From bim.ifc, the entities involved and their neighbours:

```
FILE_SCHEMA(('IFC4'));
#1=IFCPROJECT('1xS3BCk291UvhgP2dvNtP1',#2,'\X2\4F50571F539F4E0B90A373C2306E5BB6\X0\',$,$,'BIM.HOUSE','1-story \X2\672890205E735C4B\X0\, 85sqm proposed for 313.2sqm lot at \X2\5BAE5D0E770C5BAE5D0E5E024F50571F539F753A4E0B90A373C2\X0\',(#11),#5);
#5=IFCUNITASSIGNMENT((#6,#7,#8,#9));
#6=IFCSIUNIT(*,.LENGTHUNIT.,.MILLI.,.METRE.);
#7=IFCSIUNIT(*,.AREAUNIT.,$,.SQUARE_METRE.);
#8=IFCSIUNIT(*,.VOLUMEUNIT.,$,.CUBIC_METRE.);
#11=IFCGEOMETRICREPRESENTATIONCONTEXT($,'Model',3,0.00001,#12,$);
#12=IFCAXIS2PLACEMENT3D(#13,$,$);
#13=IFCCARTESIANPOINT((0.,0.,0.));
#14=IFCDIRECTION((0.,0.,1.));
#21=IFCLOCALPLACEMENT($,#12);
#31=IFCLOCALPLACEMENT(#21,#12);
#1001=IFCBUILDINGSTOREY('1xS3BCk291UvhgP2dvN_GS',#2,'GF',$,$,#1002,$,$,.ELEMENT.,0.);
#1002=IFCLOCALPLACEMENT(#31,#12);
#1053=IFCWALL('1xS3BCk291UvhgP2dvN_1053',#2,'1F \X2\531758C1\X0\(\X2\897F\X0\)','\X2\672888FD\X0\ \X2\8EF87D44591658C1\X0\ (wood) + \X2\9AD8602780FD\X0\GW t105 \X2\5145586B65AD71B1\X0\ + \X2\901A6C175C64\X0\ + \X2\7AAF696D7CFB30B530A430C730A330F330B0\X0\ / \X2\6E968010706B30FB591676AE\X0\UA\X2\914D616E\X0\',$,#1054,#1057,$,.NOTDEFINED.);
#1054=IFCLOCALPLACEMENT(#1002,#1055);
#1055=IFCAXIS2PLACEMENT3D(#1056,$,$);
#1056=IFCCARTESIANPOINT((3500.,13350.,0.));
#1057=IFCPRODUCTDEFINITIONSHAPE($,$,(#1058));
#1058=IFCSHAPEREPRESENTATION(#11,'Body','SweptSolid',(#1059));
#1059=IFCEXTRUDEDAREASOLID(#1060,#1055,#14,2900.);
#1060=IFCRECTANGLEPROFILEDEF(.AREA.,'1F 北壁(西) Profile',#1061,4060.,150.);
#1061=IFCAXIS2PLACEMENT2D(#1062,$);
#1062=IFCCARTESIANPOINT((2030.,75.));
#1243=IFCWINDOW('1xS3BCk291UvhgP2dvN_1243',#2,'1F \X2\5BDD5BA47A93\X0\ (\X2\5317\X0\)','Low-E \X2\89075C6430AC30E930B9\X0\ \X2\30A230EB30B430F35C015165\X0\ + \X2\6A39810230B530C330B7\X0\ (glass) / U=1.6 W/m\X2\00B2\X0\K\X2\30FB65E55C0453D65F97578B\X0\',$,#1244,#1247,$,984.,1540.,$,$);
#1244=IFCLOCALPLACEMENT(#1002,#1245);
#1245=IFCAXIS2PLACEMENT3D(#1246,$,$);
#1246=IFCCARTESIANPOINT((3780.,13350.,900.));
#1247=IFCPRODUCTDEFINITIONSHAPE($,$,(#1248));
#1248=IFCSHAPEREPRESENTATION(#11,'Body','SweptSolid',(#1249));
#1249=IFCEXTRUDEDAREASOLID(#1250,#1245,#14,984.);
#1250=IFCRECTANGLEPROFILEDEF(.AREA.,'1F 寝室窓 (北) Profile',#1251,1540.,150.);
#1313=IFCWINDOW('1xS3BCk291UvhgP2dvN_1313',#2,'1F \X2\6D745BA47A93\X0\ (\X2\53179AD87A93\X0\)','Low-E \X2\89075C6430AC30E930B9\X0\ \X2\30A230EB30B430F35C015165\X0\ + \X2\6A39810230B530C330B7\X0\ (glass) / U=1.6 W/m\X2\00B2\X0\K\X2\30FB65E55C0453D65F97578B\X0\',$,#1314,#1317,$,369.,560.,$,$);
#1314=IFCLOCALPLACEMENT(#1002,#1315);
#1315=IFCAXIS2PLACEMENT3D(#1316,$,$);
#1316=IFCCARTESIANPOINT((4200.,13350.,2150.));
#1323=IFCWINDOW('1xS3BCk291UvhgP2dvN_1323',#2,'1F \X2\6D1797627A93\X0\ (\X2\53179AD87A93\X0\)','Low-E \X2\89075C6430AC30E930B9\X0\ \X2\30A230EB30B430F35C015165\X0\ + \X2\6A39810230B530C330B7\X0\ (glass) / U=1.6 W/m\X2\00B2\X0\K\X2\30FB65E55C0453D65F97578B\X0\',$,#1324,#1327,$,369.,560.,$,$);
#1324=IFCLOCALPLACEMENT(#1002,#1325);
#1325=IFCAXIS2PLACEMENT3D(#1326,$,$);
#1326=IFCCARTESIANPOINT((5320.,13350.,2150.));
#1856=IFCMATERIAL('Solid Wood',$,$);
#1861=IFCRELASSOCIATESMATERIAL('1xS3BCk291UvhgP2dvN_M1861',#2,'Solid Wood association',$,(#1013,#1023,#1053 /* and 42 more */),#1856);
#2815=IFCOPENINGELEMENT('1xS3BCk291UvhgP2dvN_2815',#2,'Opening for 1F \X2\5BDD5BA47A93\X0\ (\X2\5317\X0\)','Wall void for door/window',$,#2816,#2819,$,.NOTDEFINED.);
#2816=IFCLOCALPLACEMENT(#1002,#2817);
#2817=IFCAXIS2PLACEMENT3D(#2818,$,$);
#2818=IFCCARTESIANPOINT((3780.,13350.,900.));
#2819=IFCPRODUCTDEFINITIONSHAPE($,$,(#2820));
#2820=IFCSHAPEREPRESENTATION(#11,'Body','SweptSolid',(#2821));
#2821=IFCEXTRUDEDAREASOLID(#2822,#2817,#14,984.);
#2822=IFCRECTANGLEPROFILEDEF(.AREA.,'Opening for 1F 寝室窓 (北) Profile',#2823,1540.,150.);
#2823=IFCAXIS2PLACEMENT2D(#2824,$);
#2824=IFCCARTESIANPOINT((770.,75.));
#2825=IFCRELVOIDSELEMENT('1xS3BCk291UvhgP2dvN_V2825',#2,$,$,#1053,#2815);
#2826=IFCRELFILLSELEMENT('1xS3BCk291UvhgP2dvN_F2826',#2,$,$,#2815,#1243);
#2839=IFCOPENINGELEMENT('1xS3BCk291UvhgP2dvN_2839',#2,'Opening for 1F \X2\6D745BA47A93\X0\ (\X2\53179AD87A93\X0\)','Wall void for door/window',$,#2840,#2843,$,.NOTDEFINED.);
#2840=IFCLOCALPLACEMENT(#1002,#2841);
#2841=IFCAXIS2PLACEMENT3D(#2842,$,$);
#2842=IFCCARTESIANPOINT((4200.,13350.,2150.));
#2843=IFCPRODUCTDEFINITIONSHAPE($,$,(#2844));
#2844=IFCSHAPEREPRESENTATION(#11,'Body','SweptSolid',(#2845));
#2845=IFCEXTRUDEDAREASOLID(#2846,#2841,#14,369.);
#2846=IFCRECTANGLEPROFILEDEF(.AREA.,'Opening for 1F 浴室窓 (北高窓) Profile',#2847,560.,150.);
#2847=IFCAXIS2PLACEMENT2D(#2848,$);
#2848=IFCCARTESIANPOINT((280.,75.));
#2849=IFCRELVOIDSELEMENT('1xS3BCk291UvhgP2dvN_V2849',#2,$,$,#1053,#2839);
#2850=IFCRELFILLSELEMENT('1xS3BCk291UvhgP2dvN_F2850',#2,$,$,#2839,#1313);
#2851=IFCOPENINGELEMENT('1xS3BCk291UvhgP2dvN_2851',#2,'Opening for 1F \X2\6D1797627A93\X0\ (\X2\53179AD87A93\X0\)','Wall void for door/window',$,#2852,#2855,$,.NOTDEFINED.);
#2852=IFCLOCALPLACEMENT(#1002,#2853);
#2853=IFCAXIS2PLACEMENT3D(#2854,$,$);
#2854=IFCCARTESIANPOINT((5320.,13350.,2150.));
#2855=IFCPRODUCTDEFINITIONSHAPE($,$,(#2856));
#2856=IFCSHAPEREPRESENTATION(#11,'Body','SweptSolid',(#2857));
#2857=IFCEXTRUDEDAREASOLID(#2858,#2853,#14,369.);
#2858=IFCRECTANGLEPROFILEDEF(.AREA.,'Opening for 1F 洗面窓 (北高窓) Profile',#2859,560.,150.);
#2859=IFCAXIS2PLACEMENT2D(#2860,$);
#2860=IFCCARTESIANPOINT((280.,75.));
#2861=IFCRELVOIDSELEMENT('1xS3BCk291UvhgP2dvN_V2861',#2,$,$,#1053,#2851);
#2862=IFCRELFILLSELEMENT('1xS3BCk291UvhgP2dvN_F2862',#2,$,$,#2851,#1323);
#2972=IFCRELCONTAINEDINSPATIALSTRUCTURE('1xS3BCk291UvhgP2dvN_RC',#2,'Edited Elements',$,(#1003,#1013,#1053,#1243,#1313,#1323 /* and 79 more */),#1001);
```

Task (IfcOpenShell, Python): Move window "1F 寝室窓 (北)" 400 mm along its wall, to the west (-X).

```python
import ifcopenshell
import ifcopenshell.api.geometry
import ifcopenshell.util.placement

model = ifcopenshell.open("bim.ifc")

window = model.by_guid("1xS3BCk291UvhgP2dvN_1243")
opening = window.FillsVoids[0].RelatingOpeningElement
wall = opening.VoidsElements[0].RelatingBuildingElement

wall_matrix = ifcopenshell.util.placement.get_local_placement(wall.ObjectPlacement)
shift = wall_matrix[:3, 0] * -400.0
before = ifcopenshell.util.placement.get_local_placement(window.ObjectPlacement)[:3, 3].copy()

# The window is not placed relative to its opening, so move both.
for product in (opening, window):
    matrix = ifcopenshell.util.placement.get_local_placement(product.ObjectPlacement)
    matrix[:3, 3] += shift
    ifcopenshell.api.geometry.edit_object_placement(model, product=product, matrix=matrix, is_si=False)

after = ifcopenshell.util.placement.get_local_placement(window.ObjectPlacement)[:3, 3]
print("window moved by", (after - before).round(3) + 0.0)

model.write("bim_edited.ifc")
```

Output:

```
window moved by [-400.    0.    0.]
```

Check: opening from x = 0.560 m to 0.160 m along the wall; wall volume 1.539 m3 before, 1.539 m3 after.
